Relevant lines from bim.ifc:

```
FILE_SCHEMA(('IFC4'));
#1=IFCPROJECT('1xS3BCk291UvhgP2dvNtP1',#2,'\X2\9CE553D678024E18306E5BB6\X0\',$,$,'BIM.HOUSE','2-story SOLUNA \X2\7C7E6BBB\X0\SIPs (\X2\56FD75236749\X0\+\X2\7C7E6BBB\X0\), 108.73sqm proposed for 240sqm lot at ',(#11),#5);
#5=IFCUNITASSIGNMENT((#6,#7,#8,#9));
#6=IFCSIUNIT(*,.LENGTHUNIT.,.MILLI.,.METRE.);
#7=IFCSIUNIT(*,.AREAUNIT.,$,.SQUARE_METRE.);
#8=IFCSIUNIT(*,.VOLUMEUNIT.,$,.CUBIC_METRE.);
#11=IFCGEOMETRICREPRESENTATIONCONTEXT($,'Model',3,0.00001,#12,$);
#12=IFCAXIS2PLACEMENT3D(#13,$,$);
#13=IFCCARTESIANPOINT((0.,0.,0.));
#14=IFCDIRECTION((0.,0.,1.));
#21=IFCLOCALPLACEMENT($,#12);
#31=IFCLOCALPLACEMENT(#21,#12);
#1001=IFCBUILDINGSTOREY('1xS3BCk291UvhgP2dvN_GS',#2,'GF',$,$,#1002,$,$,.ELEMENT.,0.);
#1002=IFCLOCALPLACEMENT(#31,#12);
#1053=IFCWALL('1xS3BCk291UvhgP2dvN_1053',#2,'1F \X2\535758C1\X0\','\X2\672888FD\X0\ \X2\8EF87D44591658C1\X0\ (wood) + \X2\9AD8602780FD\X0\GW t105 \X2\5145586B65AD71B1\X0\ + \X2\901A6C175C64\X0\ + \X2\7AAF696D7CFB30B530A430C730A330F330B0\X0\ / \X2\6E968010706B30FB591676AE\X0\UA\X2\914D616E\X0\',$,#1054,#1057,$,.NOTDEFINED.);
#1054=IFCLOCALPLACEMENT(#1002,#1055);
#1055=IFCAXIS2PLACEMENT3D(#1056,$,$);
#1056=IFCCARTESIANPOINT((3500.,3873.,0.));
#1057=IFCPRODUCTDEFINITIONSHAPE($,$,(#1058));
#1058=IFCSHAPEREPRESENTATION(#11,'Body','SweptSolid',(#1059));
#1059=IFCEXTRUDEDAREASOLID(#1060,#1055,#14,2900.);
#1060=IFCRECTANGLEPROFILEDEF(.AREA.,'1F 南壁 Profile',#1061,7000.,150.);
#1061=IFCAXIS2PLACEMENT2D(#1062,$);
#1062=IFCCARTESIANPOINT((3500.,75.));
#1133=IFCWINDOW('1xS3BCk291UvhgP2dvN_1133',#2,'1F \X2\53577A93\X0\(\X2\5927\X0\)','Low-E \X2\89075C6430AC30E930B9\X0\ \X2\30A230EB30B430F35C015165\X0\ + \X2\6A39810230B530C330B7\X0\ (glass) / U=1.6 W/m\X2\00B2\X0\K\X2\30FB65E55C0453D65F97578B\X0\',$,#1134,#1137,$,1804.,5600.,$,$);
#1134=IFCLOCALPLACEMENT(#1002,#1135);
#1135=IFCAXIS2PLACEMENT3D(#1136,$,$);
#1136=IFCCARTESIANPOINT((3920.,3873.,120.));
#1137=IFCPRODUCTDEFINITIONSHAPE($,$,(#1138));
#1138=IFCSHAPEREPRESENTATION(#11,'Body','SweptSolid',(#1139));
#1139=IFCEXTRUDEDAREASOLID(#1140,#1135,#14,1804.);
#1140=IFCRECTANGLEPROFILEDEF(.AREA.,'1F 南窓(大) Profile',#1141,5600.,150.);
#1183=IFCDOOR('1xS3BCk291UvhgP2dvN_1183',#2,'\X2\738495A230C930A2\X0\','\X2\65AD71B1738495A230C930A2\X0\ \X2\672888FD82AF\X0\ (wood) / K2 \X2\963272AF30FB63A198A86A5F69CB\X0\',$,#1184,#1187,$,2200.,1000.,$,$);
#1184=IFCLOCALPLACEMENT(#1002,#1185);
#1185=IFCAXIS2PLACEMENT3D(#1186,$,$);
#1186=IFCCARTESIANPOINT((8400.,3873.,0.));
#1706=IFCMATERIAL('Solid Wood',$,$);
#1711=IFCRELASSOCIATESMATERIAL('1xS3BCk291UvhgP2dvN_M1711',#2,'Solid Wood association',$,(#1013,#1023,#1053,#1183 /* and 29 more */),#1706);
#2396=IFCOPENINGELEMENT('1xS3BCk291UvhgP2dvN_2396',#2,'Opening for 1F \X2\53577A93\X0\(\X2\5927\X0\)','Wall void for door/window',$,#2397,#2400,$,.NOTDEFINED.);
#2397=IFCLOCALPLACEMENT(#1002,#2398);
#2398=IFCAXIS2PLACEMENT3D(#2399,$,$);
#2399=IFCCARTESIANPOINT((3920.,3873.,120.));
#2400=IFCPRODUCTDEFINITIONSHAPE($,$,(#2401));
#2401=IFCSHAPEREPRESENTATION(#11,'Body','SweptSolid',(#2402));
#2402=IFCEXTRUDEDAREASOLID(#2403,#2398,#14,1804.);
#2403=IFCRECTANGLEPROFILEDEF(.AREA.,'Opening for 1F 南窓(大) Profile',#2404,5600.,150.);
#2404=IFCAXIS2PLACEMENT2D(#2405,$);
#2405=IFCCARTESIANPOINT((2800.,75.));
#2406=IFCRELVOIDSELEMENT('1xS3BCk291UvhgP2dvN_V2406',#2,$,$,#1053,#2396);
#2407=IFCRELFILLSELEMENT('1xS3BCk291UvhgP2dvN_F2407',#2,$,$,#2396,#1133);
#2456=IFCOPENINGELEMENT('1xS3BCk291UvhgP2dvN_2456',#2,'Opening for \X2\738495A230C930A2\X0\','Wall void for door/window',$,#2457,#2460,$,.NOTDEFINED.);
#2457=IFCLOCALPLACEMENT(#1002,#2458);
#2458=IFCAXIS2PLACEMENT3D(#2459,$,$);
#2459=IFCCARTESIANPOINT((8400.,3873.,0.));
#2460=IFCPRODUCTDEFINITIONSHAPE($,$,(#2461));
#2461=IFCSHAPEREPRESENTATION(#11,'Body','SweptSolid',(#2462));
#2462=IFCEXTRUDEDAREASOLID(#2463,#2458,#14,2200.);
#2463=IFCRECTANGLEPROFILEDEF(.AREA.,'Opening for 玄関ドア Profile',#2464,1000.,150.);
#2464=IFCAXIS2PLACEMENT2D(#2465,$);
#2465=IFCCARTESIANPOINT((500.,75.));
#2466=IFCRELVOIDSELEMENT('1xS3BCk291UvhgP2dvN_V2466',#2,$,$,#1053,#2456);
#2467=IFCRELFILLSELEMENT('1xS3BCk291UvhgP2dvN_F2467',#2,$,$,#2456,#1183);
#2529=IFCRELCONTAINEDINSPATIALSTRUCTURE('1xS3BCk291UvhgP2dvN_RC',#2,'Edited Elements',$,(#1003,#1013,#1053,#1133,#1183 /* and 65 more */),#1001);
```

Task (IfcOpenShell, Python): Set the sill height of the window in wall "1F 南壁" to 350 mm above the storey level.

```python
import numpy as np
import ifcopenshell
import ifcopenshell.api.geometry
import ifcopenshell.geom
import ifcopenshell.util.element
import ifcopenshell.util.placement
import ifcopenshell.util.shape
import ifcopenshell.util.unit

model = ifcopenshell.open("bim.ifc")
unit_scale = ifcopenshell.util.unit.calculate_unit_scale(model)

window = model.by_guid("1xS3BCk291UvhgP2dvN_1133")
opening = window.FillsVoids[0].RelatingOpeningElement
storey = ifcopenshell.util.element.get_container(window, ifc_class="IfcBuildingStorey")
level = ifcopenshell.util.placement.get_local_placement(storey.ObjectPlacement)[2, 3]

# The opening's origin need not be at the sill, so measure its lowest point.
shape = ifcopenshell.geom.create_shape(ifcopenshell.geom.settings(), opening)
bottom = ifcopenshell.util.shape.get_shape_bottom_elevation(shape, shape.geometry) / unit_scale
dz = level + 0.35 / unit_scale - bottom

shift = np.array([0.0, 0.0, dz])
# The window is not placed relative to its opening, so move both.
for product in (opening, window):
    matrix = ifcopenshell.util.placement.get_local_placement(product.ObjectPlacement)
    matrix[:3, 3] += shift
    ifcopenshell.api.geometry.edit_object_placement(model, product=product, matrix=matrix, is_si=False)

print(f"moved by {dz * unit_scale:+.3f} m")

model.write("bim_updated.ifc")
```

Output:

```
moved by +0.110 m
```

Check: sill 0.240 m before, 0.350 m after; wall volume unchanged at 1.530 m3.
